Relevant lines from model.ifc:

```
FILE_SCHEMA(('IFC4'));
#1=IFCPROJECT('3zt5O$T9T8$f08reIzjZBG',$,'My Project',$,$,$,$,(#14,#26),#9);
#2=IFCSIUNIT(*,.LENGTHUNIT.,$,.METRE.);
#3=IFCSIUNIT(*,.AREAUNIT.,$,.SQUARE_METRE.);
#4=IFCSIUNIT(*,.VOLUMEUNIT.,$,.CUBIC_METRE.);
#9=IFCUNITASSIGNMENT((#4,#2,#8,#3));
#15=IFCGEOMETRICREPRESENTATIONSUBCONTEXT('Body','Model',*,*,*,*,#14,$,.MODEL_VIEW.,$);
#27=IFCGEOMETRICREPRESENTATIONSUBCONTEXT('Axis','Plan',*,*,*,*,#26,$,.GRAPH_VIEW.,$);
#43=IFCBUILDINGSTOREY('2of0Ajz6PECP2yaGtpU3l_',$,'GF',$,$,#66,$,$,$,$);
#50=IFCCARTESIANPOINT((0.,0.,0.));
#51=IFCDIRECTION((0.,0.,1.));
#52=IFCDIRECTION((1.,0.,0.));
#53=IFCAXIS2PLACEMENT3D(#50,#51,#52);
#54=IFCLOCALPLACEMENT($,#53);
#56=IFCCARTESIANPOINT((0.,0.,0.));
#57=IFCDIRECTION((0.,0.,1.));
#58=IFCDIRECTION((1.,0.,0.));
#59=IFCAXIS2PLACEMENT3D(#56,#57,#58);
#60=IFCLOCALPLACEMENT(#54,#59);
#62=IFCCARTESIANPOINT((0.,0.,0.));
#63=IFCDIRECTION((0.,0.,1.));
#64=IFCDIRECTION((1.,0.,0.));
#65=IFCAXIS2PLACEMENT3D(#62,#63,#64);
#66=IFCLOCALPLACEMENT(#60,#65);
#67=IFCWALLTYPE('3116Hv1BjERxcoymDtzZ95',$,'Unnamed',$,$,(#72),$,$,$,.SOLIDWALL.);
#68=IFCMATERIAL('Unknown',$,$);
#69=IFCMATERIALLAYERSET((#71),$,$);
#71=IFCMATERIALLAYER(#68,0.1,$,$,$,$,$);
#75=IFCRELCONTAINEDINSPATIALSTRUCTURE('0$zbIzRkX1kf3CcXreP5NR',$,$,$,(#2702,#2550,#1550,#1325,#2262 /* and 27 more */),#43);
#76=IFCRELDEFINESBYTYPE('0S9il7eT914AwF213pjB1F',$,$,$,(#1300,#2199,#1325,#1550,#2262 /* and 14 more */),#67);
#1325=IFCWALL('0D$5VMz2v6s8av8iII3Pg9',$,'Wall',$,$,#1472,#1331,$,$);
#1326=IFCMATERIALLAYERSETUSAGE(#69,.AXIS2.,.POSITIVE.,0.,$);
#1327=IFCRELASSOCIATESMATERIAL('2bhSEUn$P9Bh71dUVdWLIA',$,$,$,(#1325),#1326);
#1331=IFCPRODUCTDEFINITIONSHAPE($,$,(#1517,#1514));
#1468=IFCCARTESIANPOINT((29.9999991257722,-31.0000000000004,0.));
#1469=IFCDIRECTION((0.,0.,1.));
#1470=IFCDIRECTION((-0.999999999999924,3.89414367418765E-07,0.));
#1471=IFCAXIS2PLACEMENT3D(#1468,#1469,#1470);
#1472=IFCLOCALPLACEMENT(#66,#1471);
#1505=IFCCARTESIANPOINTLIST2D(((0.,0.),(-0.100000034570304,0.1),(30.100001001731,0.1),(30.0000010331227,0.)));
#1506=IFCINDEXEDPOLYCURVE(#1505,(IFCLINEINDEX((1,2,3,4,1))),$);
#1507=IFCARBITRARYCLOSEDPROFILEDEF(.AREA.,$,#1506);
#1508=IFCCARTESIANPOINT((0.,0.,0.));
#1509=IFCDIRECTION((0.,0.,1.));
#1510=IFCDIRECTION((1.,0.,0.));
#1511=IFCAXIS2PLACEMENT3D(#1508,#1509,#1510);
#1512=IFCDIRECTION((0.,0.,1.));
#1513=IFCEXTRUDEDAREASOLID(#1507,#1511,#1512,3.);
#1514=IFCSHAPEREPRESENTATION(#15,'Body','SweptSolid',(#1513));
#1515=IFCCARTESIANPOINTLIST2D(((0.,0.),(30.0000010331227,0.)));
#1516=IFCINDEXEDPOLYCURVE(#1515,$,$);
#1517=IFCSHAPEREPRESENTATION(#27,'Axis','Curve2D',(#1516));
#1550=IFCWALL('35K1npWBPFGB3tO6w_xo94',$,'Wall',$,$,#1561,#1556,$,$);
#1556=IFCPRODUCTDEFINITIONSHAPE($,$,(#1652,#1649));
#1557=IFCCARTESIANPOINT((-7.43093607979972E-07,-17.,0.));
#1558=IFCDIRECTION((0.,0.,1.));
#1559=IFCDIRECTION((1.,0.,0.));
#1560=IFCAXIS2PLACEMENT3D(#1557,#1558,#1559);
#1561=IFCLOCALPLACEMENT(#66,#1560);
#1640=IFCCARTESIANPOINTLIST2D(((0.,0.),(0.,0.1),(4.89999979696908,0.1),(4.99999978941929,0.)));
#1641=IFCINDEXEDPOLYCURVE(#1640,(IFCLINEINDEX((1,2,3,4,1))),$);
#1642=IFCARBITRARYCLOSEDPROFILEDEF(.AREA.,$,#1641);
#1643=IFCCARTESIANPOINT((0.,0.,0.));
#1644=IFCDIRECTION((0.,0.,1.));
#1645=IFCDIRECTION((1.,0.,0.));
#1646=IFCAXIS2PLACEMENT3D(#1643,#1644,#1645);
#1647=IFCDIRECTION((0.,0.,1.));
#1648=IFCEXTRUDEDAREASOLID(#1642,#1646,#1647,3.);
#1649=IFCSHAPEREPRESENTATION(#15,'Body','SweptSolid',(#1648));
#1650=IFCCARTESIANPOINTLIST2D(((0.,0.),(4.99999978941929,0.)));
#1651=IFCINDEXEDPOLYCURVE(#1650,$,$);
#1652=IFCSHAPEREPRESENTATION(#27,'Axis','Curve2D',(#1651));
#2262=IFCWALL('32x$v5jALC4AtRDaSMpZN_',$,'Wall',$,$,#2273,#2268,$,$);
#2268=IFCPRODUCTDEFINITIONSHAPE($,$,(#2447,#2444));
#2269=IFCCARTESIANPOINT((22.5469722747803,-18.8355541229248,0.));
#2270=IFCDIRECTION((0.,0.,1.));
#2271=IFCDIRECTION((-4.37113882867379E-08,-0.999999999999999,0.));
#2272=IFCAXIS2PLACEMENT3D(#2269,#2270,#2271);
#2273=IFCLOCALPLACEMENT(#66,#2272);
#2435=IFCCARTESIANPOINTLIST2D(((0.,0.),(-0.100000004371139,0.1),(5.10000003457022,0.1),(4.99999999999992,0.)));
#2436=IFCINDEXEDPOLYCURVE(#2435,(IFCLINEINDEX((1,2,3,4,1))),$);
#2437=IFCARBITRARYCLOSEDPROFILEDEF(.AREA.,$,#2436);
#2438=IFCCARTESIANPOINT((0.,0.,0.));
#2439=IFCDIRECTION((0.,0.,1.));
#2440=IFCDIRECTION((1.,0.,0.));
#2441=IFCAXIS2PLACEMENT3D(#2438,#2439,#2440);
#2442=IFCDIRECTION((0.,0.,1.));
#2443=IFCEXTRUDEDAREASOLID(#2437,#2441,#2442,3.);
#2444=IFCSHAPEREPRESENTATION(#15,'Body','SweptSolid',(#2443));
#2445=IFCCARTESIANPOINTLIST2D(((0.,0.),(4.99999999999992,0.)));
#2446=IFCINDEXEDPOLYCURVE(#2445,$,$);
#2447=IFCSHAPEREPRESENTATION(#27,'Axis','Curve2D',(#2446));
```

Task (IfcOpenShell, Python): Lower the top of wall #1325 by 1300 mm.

```python
import ifcopenshell
import ifcopenshell.geom
import ifcopenshell.util.representation
import ifcopenshell.util.shape
import ifcopenshell.util.unit

model = ifcopenshell.open("model.ifc")
unit_scale = ifcopenshell.util.unit.calculate_unit_scale(model)
settings = ifcopenshell.geom.settings()


def volume(element):
    """Net volume in cubic metres, openings subtracted."""
    shape = ifcopenshell.geom.create_shape(settings, element)
    return ifcopenshell.util.shape.get_volume(shape.geometry)


wall = model.by_id(1325)
before = volume(wall)

body = ifcopenshell.util.representation.get_representation(wall, "Model", "Body")
solid = body.Items[0]
old_height = solid.Depth
solid.Depth -= 1.3 / unit_scale
after = volume(wall)

print(f"height {old_height:g} -> {solid.Depth:g}, volume {before:.3f} -> {after:.3f} m3")

model.write("model_updated.ifc")
```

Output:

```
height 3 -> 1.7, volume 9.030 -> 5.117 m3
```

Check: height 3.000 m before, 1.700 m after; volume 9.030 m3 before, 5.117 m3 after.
